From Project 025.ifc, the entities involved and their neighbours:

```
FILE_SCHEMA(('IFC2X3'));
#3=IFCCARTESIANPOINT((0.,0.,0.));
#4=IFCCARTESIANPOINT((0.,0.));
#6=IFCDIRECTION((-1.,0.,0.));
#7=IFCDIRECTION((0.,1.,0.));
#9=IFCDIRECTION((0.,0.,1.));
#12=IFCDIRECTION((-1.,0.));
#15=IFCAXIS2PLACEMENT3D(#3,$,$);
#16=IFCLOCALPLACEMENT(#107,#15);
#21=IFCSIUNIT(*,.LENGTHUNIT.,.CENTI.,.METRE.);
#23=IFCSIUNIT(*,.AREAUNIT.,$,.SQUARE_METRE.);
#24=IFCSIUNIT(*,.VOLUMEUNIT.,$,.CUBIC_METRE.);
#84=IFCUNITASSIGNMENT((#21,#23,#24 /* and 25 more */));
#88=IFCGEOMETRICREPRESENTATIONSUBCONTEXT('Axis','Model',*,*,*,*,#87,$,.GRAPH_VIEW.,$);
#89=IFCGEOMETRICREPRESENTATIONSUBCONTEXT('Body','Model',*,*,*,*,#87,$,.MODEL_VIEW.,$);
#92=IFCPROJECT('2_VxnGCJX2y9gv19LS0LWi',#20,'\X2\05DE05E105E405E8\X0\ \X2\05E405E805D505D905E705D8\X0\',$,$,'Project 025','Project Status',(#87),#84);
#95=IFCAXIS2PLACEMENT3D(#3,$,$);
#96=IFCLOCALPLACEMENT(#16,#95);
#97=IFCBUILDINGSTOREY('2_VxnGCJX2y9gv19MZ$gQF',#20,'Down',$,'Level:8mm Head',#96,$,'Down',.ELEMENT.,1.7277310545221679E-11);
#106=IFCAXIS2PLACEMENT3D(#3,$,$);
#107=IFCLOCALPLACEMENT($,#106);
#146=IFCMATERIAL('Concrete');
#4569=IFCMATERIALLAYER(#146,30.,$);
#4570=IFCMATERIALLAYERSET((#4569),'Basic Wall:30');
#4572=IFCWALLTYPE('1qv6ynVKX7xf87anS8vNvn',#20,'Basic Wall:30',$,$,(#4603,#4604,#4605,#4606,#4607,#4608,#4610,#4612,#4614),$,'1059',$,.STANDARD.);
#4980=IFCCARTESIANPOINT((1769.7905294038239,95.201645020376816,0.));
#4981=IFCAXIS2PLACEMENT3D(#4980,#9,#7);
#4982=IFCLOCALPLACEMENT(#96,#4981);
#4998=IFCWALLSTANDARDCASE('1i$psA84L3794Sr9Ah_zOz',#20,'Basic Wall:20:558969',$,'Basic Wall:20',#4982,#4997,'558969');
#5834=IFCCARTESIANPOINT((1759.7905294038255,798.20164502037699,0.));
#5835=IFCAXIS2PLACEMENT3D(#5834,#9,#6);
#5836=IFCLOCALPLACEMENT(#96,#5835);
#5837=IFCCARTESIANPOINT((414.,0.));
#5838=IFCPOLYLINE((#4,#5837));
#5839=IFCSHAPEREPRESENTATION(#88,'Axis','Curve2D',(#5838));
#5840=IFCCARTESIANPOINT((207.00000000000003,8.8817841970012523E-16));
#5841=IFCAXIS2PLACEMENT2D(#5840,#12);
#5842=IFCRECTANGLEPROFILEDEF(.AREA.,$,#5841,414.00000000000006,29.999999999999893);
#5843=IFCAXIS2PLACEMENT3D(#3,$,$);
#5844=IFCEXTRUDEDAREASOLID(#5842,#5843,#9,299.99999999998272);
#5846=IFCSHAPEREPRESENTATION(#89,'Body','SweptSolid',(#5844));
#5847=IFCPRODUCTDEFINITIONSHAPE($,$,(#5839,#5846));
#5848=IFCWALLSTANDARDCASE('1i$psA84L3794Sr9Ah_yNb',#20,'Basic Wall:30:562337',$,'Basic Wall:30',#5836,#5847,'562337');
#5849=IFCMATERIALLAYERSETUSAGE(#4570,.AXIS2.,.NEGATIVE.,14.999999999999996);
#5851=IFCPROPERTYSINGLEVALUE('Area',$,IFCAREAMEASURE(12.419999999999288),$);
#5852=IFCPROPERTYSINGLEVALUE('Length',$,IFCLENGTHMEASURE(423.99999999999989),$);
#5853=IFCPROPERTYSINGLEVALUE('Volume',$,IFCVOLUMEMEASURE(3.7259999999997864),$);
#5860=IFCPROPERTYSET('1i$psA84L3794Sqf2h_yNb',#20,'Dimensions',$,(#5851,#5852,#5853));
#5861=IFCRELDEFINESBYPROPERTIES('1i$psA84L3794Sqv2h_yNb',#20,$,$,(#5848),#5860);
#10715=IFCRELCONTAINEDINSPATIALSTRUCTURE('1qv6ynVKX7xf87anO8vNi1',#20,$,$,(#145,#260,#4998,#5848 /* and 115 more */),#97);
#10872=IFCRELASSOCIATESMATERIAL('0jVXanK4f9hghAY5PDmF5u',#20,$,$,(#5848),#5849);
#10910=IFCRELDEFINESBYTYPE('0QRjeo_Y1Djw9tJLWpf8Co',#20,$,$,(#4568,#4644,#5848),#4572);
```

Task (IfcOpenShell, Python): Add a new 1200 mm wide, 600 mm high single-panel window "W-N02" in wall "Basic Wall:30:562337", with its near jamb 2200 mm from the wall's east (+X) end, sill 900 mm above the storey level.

```python
import numpy as np
import ifcopenshell
import ifcopenshell.api.feature
import ifcopenshell.api.geometry
import ifcopenshell.api.pset
import ifcopenshell.api.root
import ifcopenshell.api.spatial
import ifcopenshell.api.type
import ifcopenshell.geom
import ifcopenshell.util.element
import ifcopenshell.util.placement
import ifcopenshell.util.representation
import ifcopenshell.util.shape
import ifcopenshell.util.unit

model = ifcopenshell.open("Project 025.ifc")
unit_scale = ifcopenshell.util.unit.calculate_unit_scale(model)
area_scale = ifcopenshell.util.unit.calculate_unit_scale(model, "AREAUNIT")
volume_scale = ifcopenshell.util.unit.calculate_unit_scale(model, "VOLUMEUNIT")
settings = ifcopenshell.geom.settings()


def volume(element):
    """Net volume in cubic metres, openings subtracted."""
    shape = ifcopenshell.geom.create_shape(settings, element)
    return ifcopenshell.util.shape.get_volume(shape.geometry)


wall = model.by_id(5848)
storey = ifcopenshell.util.element.get_container(wall, ifc_class="IfcBuildingStorey")
context = ifcopenshell.util.representation.get_context(model, "Model", "Body", "MODEL_VIEW")
before = volume(wall)

width, height, from_end, sill = 1.2, 0.6, 2.2, 0.9  # metres

# The wall runs along its own X axis, and the end named is its -X end.
wall_shape = ifcopenshell.geom.create_shape(settings, wall)
x, y, z = ifcopenshell.util.shape.get_vertices(wall_shape.geometry).T
start = x.min() + from_end
face, thickness = float(y.min()), float(y.max() - y.min())
wall_matrix = ifcopenshell.util.placement.get_local_placement(wall.ObjectPlacement)
level = ifcopenshell.util.placement.get_local_placement(storey.ObjectPlacement)[2, 3]


def in_wall(x, y):
    """Placement at x, y metres in the wall's axes, at sill height."""
    matrix = wall_matrix.copy()
    matrix[:, 3] = wall_matrix @ np.array([x / unit_scale, y / unit_scale, 0.0, 1.0])
    matrix[2, 3] = level + sill / unit_scale
    return matrix


# Opening: a box that overshoots both wall faces by 50 mm.
opening = ifcopenshell.api.root.create_entity(model, ifc_class="IfcOpeningElement")
box = ifcopenshell.api.geometry.add_wall_representation(
    model, context=context, length=width, height=height, thickness=thickness + 0.1
)
ifcopenshell.api.geometry.assign_representation(model, product=opening, representation=box)
ifcopenshell.api.geometry.edit_object_placement(model, product=opening, matrix=in_wall(start, face - 0.05), is_si=False)
ifcopenshell.api.feature.add_feature(model, feature=opening, element=wall)

window = ifcopenshell.api.root.create_entity(model, ifc_class="IfcWindow", name="W-N02")
window.OverallWidth, window.OverallHeight = width / unit_scale, height / unit_scale
body = ifcopenshell.api.geometry.add_window_representation(
    model,
    context=context,
    overall_width=window.OverallWidth,
    overall_height=window.OverallHeight,
    partition_type="SINGLE_PANEL",
)
ifcopenshell.api.geometry.assign_representation(model, product=window, representation=body)
ifcopenshell.api.spatial.assign_container(model, products=[window], relating_structure=storey)
fills = ifcopenshell.api.feature.add_filling(model, opening=opening, element=window)
fills.OwnerHistory = window.OwnerHistory  # required in IFC2X3

# IFC2X3 keeps the operation on the window style.
style = ifcopenshell.api.root.create_entity(model, ifc_class="IfcWindowStyle", name="W-N02")
style.OperationType, style.ConstructionType = "SINGLE_PANEL", "NOTDEFINED"
style.ParameterTakesPrecedence = style.Sizeable = False
ifcopenshell.api.type.assign_type(model, related_objects=[window], relating_type=style)

# Centre the window in the wall's thickness.
ifcopenshell.api.geometry.edit_object_placement(model, product=window, matrix=in_wall(start, face), is_si=False)
window_shape = ifcopenshell.geom.create_shape(settings, window)
depth = ifcopenshell.util.shape.get_vertices(window_shape.geometry)[:, 1]
offset = face + thickness / 2 - (depth.min() + depth.max()) / 2
ifcopenshell.api.geometry.edit_object_placement(model, product=window, matrix=in_wall(start, offset), is_si=False)

after = volume(wall)

# Update the wall's stored quantities.
pset = model.by_id(ifcopenshell.util.element.get_pset(wall, "Dimensions", should_inherit=False)["id"])
ifcopenshell.api.pset.edit_pset(model, pset=pset, properties={
    "Area": model.create_entity("IfcAreaMeasure", after / thickness / area_scale),
    "Volume": model.create_entity("IfcVolumeMeasure", after / volume_scale),
})

print(f"wall volume {before:.3f} -> {after:.3f} m3")

model.write("Project 025_rev.ifc")
```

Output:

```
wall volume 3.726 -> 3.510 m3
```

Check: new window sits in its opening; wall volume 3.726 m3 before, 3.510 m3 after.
